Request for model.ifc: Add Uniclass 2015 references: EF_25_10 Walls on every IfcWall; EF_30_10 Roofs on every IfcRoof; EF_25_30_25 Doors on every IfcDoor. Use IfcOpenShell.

First a look at what the model holds.

```python
import ifcopenshell

model = ifcopenshell.open("model.ifc")
print(model.schema)
print("classifications:", [c.Name for c in model.by_type("IfcClassification")])
for ifc_class in ("IfcDoor", "IfcRoof", "IfcStair", "IfcWall", "IfcWindow"):
    print(ifc_class, len(model.by_type(ifc_class)))
```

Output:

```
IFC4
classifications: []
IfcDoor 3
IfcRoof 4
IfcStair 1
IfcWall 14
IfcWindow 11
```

```python
import ifcopenshell
import ifcopenshell.api.classification

model = ifcopenshell.open("model.ifc")

system = ifcopenshell.api.classification.add_classification(model, classification="Uniclass 2015")

codes = {
    "IfcWall": ("EF_25_10", "Walls"),
    "IfcRoof": ("EF_30_10", "Roofs"),
    "IfcDoor": ("EF_25_30_25", "Doors"),
}
for ifc_class, (code, name) in codes.items():
    products = model.by_type(ifc_class)
    ifcopenshell.api.classification.add_reference(
        model, products=products, classification=system, identification=code, name=name
    )
    print(code, len(products))

model.write("model_v2.ifc")
```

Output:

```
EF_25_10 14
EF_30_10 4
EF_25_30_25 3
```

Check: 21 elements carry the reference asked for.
